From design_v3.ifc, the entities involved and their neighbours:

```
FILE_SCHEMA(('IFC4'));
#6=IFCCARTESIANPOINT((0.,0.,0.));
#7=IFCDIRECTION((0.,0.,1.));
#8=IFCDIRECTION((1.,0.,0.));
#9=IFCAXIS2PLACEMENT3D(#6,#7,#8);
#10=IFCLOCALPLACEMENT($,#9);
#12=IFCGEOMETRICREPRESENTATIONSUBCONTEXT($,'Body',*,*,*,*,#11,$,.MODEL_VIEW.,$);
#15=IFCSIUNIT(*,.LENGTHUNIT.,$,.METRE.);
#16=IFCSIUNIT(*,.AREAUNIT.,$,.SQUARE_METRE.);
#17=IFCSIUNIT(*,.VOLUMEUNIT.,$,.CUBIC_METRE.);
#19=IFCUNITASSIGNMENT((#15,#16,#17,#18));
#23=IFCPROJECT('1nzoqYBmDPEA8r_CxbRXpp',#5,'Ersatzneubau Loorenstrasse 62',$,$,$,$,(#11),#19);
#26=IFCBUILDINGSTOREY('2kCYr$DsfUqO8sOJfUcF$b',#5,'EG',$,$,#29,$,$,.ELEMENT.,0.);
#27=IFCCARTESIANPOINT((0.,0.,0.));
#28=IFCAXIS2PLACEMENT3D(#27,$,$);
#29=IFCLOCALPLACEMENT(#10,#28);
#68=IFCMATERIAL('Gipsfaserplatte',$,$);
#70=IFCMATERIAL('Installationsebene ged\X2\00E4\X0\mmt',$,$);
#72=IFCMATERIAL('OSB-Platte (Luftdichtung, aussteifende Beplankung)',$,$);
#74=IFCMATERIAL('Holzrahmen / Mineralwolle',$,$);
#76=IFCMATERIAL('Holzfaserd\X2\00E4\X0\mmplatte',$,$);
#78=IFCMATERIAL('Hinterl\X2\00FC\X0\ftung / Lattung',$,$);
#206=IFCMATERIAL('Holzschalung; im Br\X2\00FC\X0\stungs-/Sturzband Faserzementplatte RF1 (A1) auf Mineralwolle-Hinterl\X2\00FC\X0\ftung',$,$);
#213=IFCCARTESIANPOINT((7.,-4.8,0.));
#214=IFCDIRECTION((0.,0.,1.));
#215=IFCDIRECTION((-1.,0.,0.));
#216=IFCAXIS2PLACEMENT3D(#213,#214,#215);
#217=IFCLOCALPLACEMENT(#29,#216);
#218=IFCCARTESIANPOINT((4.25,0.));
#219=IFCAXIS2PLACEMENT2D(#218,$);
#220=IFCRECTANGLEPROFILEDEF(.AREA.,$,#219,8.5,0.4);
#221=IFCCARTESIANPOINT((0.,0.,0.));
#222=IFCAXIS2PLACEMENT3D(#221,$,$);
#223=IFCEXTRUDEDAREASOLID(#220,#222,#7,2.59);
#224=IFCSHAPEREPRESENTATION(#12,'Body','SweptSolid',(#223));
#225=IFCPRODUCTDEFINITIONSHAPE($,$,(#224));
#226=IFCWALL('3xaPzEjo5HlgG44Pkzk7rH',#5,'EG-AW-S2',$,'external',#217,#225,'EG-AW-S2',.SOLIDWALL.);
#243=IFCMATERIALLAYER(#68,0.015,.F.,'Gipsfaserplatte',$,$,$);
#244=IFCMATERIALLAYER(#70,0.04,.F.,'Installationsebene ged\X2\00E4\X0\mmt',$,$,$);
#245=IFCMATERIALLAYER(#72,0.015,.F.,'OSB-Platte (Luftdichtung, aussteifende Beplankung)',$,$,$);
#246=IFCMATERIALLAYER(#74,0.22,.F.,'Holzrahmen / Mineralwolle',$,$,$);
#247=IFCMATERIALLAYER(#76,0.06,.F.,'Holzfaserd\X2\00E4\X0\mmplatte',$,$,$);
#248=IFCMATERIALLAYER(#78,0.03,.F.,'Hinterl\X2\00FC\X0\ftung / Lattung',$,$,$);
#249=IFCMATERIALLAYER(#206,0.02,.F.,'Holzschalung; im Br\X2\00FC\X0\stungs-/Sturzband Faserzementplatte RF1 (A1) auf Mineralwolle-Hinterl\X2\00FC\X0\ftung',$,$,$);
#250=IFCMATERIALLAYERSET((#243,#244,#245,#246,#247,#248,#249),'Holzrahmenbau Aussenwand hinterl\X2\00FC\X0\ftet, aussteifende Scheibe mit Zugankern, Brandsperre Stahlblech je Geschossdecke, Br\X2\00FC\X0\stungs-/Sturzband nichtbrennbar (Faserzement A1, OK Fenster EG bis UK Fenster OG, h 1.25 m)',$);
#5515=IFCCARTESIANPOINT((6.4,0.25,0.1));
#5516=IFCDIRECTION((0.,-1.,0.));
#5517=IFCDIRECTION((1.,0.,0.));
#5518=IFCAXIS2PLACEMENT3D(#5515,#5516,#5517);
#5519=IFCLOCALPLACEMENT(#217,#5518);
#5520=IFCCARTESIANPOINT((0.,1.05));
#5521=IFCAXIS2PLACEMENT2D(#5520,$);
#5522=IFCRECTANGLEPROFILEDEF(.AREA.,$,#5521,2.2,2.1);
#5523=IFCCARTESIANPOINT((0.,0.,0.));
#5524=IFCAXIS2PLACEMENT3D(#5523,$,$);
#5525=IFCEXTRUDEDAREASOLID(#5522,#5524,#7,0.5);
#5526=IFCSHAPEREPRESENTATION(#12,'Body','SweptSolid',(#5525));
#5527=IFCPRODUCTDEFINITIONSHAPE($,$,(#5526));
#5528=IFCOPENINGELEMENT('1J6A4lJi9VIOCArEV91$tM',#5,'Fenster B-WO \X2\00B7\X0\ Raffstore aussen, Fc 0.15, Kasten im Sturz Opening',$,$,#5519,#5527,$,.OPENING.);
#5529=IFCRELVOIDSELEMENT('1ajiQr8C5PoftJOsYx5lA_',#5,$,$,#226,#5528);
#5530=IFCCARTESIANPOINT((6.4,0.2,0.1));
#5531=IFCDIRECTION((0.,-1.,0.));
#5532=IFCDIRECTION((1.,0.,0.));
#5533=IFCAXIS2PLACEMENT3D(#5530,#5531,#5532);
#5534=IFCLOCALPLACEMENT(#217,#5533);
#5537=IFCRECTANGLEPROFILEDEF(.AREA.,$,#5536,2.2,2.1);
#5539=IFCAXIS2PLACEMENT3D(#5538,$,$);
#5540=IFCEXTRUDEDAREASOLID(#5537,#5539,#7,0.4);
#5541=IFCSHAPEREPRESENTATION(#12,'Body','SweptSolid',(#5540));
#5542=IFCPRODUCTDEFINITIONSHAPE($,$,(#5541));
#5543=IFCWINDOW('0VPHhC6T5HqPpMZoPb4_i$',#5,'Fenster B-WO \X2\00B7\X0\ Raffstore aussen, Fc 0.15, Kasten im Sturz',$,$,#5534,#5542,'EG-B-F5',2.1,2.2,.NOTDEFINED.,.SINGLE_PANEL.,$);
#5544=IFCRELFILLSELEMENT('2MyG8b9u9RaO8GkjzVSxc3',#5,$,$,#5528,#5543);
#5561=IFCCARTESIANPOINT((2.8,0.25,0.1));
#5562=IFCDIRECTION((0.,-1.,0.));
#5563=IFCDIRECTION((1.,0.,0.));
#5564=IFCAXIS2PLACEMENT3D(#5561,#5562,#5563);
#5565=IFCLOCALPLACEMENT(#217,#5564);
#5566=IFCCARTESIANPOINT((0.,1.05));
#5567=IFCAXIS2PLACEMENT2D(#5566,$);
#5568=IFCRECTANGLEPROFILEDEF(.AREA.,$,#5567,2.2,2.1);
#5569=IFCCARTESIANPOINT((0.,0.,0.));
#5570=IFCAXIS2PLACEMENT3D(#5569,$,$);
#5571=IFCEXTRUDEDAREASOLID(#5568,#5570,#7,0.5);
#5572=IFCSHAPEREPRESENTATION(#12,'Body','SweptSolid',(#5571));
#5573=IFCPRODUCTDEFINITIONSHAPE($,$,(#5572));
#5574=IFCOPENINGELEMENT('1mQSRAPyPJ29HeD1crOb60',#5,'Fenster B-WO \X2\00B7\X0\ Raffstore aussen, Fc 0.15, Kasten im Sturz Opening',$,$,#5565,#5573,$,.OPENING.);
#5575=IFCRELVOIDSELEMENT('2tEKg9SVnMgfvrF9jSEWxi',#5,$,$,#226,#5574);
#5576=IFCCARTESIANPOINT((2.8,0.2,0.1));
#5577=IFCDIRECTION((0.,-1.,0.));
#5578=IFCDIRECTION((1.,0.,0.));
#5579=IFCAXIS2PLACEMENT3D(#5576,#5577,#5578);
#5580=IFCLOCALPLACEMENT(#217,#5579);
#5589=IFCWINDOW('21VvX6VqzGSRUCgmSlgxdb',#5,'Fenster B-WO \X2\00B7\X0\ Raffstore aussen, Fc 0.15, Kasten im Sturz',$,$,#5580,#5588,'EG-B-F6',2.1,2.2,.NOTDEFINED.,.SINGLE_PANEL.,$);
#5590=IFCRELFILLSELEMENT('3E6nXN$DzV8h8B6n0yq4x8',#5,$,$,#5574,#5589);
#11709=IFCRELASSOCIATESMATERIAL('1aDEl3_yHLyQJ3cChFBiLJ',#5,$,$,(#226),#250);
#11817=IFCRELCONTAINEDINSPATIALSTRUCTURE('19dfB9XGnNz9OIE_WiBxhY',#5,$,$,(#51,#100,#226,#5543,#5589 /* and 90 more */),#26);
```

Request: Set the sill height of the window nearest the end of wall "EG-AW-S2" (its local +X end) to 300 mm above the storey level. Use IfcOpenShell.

```python
import numpy as np
import ifcopenshell
import ifcopenshell.api.geometry
import ifcopenshell.geom
import ifcopenshell.util.element
import ifcopenshell.util.placement
import ifcopenshell.util.shape
import ifcopenshell.util.unit

model = ifcopenshell.open("design_v3.ifc")
unit_scale = ifcopenshell.util.unit.calculate_unit_scale(model)

window = model.by_guid("0VPHhC6T5HqPpMZoPb4_i$")
opening = window.FillsVoids[0].RelatingOpeningElement
storey = ifcopenshell.util.element.get_container(window, ifc_class="IfcBuildingStorey")
level = ifcopenshell.util.placement.get_local_placement(storey.ObjectPlacement)[2, 3]

# The opening's origin need not be at the sill, so measure its lowest point.
shape = ifcopenshell.geom.create_shape(ifcopenshell.geom.settings(), opening)
bottom = ifcopenshell.util.shape.get_shape_bottom_elevation(shape, shape.geometry) / unit_scale
dz = level + 0.3 - bottom

shift = np.array([0.0, 0.0, dz])
# The window is not placed relative to its opening, so move both.
for product in (opening, window):
    matrix = ifcopenshell.util.placement.get_local_placement(product.ObjectPlacement)
    matrix[:3, 3] += shift
    ifcopenshell.api.geometry.edit_object_placement(model, product=product, matrix=matrix, is_si=False)

print(f"moved by {dz * unit_scale:+.3f} m")

model.write("design_v3-out.ifc")
```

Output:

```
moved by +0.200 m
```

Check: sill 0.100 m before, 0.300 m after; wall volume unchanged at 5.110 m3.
